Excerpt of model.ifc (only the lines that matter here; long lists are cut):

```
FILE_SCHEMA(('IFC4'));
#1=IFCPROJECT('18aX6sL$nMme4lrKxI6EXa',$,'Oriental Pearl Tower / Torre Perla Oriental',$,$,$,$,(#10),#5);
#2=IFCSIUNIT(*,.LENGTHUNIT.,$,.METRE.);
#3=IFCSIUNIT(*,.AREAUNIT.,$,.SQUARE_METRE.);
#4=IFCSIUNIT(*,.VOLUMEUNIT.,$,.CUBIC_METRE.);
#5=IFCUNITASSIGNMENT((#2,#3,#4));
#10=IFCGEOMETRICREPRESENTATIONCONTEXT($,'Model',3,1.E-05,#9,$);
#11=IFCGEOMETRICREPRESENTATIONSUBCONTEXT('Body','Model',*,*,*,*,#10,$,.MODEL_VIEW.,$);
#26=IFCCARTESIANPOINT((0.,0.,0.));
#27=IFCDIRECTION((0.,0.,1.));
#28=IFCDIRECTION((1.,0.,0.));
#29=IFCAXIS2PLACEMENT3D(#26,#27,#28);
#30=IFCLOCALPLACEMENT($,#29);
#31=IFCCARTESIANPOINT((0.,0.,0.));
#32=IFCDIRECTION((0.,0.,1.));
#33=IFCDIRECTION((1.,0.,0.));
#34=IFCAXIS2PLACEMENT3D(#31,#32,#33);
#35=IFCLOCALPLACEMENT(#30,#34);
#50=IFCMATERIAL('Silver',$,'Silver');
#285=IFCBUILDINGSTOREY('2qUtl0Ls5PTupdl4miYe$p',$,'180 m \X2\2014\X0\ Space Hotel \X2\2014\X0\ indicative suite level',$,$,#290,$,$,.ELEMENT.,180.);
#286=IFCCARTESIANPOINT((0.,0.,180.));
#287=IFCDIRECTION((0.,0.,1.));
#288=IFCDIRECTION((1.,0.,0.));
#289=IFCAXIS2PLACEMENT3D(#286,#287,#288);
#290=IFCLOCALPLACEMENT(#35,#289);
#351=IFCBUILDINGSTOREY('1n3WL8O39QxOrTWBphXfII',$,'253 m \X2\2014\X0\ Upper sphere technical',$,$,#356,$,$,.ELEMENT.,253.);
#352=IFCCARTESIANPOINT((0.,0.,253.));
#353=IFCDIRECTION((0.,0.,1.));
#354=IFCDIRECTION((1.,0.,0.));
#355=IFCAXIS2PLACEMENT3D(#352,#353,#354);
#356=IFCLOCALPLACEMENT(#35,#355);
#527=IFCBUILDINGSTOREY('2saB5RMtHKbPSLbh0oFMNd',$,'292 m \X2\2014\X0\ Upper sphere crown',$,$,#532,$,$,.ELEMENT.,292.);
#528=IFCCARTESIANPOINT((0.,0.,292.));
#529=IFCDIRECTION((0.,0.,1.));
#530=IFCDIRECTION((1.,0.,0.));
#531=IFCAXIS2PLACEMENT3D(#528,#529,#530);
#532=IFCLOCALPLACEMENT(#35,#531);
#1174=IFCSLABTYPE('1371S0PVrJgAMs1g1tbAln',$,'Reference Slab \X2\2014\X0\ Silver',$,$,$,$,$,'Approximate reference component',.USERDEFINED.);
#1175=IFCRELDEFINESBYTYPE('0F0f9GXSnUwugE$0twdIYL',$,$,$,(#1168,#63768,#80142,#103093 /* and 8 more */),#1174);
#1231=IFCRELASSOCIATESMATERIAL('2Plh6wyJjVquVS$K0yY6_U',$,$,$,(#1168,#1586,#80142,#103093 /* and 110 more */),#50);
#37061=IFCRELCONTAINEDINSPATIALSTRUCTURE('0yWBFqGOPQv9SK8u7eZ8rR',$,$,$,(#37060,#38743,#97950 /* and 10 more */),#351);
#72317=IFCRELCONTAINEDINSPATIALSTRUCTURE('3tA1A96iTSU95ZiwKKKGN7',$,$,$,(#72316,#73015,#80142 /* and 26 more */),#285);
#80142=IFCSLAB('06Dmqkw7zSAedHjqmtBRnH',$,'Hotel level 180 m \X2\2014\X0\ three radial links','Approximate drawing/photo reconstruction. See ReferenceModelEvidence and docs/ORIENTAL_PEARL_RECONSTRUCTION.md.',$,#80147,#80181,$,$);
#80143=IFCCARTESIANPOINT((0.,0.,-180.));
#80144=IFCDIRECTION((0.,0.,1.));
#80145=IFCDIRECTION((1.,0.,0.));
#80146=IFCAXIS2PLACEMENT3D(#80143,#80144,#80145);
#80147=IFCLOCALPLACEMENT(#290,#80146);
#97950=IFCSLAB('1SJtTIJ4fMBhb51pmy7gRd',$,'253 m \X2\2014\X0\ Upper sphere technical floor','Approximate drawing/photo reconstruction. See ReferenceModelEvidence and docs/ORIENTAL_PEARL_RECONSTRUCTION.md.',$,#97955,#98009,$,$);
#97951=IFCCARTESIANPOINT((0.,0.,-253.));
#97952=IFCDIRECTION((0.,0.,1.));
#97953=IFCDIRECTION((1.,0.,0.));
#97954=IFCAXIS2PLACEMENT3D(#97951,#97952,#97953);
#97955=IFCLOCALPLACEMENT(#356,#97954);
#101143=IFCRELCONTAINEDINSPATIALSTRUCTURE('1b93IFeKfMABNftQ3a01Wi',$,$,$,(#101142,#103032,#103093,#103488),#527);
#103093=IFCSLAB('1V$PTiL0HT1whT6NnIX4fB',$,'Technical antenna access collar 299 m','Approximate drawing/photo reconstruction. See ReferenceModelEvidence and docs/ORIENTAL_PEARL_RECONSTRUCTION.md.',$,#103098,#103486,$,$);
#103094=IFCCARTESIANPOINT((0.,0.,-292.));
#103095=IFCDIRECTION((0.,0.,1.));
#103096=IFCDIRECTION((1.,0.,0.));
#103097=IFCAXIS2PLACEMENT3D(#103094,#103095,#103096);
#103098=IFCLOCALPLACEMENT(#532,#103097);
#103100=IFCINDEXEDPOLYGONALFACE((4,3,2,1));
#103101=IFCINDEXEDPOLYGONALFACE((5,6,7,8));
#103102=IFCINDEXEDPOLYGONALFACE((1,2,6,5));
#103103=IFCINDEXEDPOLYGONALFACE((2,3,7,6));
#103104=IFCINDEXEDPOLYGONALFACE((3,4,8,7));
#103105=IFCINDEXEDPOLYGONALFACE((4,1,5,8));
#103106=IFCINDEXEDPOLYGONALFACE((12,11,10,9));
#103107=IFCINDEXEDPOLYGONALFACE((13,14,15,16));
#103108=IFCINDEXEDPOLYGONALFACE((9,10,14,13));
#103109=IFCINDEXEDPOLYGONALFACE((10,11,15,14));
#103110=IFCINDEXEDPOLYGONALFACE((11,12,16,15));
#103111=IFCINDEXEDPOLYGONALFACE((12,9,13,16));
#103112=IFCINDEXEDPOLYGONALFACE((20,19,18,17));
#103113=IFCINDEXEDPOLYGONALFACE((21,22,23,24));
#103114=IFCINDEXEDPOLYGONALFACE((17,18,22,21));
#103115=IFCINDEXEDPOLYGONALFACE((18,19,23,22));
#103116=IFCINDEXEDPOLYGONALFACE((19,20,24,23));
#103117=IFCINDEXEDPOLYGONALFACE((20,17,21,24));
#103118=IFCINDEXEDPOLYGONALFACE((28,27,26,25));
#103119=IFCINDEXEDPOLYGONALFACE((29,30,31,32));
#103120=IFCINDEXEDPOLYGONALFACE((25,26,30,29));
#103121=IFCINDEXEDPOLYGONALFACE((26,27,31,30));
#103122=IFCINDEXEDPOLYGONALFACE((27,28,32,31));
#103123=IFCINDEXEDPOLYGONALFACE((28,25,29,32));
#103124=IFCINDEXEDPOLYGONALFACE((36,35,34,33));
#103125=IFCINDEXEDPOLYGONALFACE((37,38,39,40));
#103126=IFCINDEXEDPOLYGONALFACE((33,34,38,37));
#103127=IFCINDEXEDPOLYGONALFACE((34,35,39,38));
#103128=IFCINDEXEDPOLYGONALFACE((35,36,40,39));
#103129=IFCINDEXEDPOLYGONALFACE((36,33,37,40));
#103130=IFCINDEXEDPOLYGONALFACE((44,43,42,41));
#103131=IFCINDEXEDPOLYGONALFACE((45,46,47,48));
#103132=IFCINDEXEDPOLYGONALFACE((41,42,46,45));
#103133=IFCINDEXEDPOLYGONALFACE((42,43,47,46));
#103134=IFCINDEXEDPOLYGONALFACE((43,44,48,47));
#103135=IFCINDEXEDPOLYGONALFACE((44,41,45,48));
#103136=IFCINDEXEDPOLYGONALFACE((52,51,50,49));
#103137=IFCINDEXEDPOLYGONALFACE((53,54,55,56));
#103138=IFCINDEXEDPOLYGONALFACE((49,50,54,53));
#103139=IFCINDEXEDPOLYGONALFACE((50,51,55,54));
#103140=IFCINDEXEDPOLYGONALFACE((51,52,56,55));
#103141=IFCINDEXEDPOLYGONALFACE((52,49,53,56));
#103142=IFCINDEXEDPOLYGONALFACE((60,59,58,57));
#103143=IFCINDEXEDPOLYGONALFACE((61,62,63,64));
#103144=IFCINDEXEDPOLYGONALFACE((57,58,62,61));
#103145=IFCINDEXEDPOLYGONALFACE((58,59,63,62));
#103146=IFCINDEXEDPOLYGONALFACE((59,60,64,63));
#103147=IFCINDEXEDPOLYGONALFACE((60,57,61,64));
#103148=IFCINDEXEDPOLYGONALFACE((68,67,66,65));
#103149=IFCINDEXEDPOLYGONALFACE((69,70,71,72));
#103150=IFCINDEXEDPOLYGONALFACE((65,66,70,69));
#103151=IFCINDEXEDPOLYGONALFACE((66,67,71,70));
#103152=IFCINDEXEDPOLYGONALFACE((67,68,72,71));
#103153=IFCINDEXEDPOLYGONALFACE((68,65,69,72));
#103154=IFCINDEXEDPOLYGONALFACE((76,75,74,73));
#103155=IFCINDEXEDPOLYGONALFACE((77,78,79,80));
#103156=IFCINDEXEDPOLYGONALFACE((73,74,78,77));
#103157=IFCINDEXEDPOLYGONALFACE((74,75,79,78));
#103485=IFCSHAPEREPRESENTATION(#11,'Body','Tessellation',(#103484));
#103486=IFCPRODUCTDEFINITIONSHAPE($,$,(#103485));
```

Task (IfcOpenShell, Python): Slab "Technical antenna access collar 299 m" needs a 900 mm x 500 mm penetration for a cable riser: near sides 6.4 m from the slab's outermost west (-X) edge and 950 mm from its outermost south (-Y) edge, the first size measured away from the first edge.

```python
import numpy as np
import ifcopenshell
import ifcopenshell.api.feature
import ifcopenshell.api.geometry
import ifcopenshell.api.root
import ifcopenshell.geom
import ifcopenshell.util.placement
import ifcopenshell.util.representation
import ifcopenshell.util.shape
import ifcopenshell.util.unit

model = ifcopenshell.open("model.ifc")
unit_scale = ifcopenshell.util.unit.calculate_unit_scale(model)
settings = ifcopenshell.geom.settings()


def volume(element):
    """Net volume in cubic metres, openings subtracted."""
    shape = ifcopenshell.geom.create_shape(settings, element)
    return ifcopenshell.util.shape.get_volume(shape.geometry)


slab = model.by_id(103093)
before = volume(slab)

# Extent in the slab's own axes, in metres. The edges named are its -X and -Y sides.
slab_shape = ifcopenshell.geom.create_shape(settings, slab)
vertices = ifcopenshell.util.shape.get_vertices(slab_shape.geometry)
x_min, y_min, bottom = vertices.min(axis=0)
top = vertices[:, 2].max()

opening = ifcopenshell.api.root.create_entity(model, ifc_class="IfcOpeningElement", name="Cable riser opening", predefined_type="OPENING")
context = ifcopenshell.util.representation.get_context(model, "Model", "Body", "MODEL_VIEW")
width, depth = 0.9, 0.5
outline = [(0.0, 0.0), (width, 0.0), (width, depth), (0.0, depth), (0.0, 0.0)]
# Overshoot both faces by 50 mm so the cut is clean.
shape = ifcopenshell.api.geometry.add_slab_representation(
    model, context=context, depth=top - bottom + 0.1, polyline=outline
)
ifcopenshell.api.geometry.assign_representation(model, product=opening, representation=shape)

matrix = ifcopenshell.util.placement.get_local_placement(slab.ObjectPlacement)
matrix[:, 3] = matrix @ np.append(np.array([x_min + 6.4, y_min + 0.95, bottom - 0.05]) / unit_scale, 1.0)
ifcopenshell.api.geometry.edit_object_placement(model, product=opening, matrix=matrix, is_si=False)
ifcopenshell.api.feature.add_feature(model, feature=opening, element=slab)

after = volume(slab)

print(f"slab volume {before:.3f} -> {after:.3f} m3")

model.write("model_v2.ifc")
```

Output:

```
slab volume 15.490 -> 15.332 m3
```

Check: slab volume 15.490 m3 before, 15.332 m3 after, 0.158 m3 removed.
